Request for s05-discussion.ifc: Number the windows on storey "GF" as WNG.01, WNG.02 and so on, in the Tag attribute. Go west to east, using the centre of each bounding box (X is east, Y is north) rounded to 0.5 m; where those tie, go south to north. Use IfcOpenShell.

First a look at what the model holds.

```python
import ifcopenshell
import ifcopenshell.util.element
import ifcopenshell.util.placement

model = ifcopenshell.open("s05-discussion.ifc")
print(model.schema)
storey = next(s for s in model.by_type("IfcBuildingStorey") if s.Name == "GF")
windows = [e for e in ifcopenshell.util.element.get_decomposition(storey) if e.is_a("IfcWindow")]
for e in sorted(windows, key=lambda e: e.id()):
    origin = ifcopenshell.util.placement.get_local_placement(e.ObjectPlacement)[:3, 3]
    print(e.id(), e.Tag, e.Name, origin.round(2) + 0.0, sep=" | ")
```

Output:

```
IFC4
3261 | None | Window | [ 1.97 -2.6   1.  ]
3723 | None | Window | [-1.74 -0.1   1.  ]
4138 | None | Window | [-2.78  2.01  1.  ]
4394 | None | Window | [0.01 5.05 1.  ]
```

```python
import ifcopenshell
import ifcopenshell.geom
import ifcopenshell.util.element
import ifcopenshell.util.shape

model = ifcopenshell.open("s05-discussion.ifc")
settings = ifcopenshell.geom.settings()
settings.set("use-world-coords", True)


def centre(element):
    shape = ifcopenshell.geom.create_shape(settings, element)
    return ifcopenshell.util.shape.get_bbox_centroid(shape.geometry)


storey = next(s for s in model.by_type("IfcBuildingStorey") if s.Name == "GF")
windows = [e for e in ifcopenshell.util.element.get_decomposition(storey) if e.is_a("IfcWindow")]

# Insertion points can sit at a corner or the storey origin, so sort by the geometry (in metres).
centres = {e: centre(e) for e in windows}
windows.sort(key=lambda e: (round(centres[e][0] / 0.5), centres[e][1]))

for i, e in enumerate(windows, start=1):
    number = f"WNG.{i:02d}"
    e.Tag = number
    print(e.id(), number)

model.write("s05-discussion-out.ifc")
```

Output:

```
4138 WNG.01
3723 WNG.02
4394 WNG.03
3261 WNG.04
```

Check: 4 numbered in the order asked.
